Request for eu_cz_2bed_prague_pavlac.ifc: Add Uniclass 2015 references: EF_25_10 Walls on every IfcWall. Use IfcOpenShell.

First a look at what the model holds.

```python
import ifcopenshell

model = ifcopenshell.open("eu_cz_2bed_prague_pavlac.ifc")
print(model.schema)
print("classifications:", [c.Name for c in model.by_type("IfcClassification")])
for ifc_class in ("IfcDoor", "IfcRoof", "IfcStair", "IfcWall", "IfcWindow"):
    print(ifc_class, len(model.by_type(ifc_class)))
```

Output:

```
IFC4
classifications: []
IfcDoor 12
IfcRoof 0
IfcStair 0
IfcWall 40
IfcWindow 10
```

```python
import ifcopenshell
import ifcopenshell.api.classification

model = ifcopenshell.open("eu_cz_2bed_prague_pavlac.ifc")

system = ifcopenshell.api.classification.add_classification(model, classification="Uniclass 2015")

codes = {
    "IfcWall": ("EF_25_10", "Walls"),
}
for ifc_class, (code, name) in codes.items():
    products = model.by_type(ifc_class)
    ifcopenshell.api.classification.add_reference(
        model, products=products, classification=system, identification=code, name=name
    )
    print(code, len(products))

model.write("eu_cz_2bed_prague_pavlac-out.ifc")
```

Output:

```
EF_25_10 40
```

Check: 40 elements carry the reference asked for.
